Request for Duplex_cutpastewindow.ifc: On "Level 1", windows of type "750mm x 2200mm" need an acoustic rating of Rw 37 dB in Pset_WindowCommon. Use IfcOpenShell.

First a look at what the model holds.

```python
import ifcopenshell
import ifcopenshell.util.element

model = ifcopenshell.open("Duplex_cutpastewindow.ifc")
print(model.schema)
storey = next(s for s in model.by_type("IfcBuildingStorey") if s.Name == "Level 1")
windows = [e for e in ifcopenshell.util.element.get_decomposition(storey) if e.is_a("IfcWindow")]
seen = {}
for e in windows:
    element_type = ifcopenshell.util.element.get_type(e)
    key = (element_type.Name if element_type != e and element_type else None, ifcopenshell.util.element.get_pset(e, "Pset_WindowCommon", "AcousticRating"))
    seen[key] = seen.get(key, 0) + 1
for (name, value), count in sorted(seen.items(), key=str):
    print(count, "x", name, "|", value)
```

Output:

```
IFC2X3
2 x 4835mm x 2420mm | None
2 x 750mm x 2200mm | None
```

```python
import ifcopenshell
import ifcopenshell.api.pset
import ifcopenshell.util.element

model = ifcopenshell.open("Duplex_cutpastewindow.ifc")

storey = next(s for s in model.by_type("IfcBuildingStorey") if s.Name == "Level 1")
windows = [e for e in ifcopenshell.util.element.get_decomposition(storey) if e.is_a("IfcWindow")]

count = 0
for e in windows:
    element_type = ifcopenshell.util.element.get_type(e)
    if element_type in (None, e) or element_type.Name != "750mm x 2200mm":
        continue
    # add_pset returns the element's existing set when there is one.
    pset = ifcopenshell.api.pset.add_pset(model, product=e, name="Pset_WindowCommon")
    ifcopenshell.api.pset.edit_pset(model, pset=pset, properties={"AcousticRating": "Rw 37 dB"})
    count += 1

print(count, "windows updated")

model.write("Duplex_cutpastewindow_rev.ifc")
```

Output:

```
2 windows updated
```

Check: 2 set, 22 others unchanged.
